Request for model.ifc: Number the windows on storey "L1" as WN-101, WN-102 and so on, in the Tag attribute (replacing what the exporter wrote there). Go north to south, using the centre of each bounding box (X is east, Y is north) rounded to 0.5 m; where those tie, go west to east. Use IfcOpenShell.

First a look at what the model holds.

```python
import ifcopenshell
import ifcopenshell.util.element
import ifcopenshell.util.placement

model = ifcopenshell.open("model.ifc")
print(model.schema)
storey = next(s for s in model.by_type("IfcBuildingStorey") if s.Name == "L1")
windows = [e for e in ifcopenshell.util.element.get_decomposition(storey) if e.is_a("IfcWindow")]
for e in sorted(windows, key=lambda e: e.id()):
    origin = ifcopenshell.util.placement.get_local_placement(e.ObjectPlacement)[:3, 3]
    print(e.id(), e.Tag, e.Name, origin.round(2) + 0.0, sep=" | ")
```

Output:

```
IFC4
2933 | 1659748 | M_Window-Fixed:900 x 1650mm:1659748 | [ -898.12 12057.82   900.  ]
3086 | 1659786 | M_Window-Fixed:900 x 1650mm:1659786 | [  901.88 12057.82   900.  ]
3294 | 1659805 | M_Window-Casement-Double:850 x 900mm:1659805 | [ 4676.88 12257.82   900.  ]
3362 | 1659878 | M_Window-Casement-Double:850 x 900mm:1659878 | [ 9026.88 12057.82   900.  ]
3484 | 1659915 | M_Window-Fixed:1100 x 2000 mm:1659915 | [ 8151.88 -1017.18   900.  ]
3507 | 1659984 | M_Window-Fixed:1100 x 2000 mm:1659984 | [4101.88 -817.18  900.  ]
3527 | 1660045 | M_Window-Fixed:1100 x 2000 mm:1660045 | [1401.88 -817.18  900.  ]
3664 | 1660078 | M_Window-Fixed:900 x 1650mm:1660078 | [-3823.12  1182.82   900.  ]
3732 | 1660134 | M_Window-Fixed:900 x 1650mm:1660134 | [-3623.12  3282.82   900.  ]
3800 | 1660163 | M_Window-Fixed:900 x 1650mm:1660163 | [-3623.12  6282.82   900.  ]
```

```python
import ifcopenshell
import ifcopenshell.geom
import ifcopenshell.util.element
import ifcopenshell.util.shape

model = ifcopenshell.open("model.ifc")
settings = ifcopenshell.geom.settings()
settings.set("use-world-coords", True)


def centre(element):
    shape = ifcopenshell.geom.create_shape(settings, element)
    return ifcopenshell.util.shape.get_bbox_centroid(shape.geometry)


storey = next(s for s in model.by_type("IfcBuildingStorey") if s.Name == "L1")
windows = [e for e in ifcopenshell.util.element.get_decomposition(storey) if e.is_a("IfcWindow")]

# Insertion points can sit at a corner or the storey origin, so sort by the geometry (in metres).
centres = {e: centre(e) for e in windows}
windows.sort(key=lambda e: (-round(centres[e][1] / 0.5), centres[e][0]))

for i, e in enumerate(windows, start=1):
    number = f"WN-1{i:02d}"
    e.Tag = number
    print(e.id(), number)

model.write("model_v2.ifc")
```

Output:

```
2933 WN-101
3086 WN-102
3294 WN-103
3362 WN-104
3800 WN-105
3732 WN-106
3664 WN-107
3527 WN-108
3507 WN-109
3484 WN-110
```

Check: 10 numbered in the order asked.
